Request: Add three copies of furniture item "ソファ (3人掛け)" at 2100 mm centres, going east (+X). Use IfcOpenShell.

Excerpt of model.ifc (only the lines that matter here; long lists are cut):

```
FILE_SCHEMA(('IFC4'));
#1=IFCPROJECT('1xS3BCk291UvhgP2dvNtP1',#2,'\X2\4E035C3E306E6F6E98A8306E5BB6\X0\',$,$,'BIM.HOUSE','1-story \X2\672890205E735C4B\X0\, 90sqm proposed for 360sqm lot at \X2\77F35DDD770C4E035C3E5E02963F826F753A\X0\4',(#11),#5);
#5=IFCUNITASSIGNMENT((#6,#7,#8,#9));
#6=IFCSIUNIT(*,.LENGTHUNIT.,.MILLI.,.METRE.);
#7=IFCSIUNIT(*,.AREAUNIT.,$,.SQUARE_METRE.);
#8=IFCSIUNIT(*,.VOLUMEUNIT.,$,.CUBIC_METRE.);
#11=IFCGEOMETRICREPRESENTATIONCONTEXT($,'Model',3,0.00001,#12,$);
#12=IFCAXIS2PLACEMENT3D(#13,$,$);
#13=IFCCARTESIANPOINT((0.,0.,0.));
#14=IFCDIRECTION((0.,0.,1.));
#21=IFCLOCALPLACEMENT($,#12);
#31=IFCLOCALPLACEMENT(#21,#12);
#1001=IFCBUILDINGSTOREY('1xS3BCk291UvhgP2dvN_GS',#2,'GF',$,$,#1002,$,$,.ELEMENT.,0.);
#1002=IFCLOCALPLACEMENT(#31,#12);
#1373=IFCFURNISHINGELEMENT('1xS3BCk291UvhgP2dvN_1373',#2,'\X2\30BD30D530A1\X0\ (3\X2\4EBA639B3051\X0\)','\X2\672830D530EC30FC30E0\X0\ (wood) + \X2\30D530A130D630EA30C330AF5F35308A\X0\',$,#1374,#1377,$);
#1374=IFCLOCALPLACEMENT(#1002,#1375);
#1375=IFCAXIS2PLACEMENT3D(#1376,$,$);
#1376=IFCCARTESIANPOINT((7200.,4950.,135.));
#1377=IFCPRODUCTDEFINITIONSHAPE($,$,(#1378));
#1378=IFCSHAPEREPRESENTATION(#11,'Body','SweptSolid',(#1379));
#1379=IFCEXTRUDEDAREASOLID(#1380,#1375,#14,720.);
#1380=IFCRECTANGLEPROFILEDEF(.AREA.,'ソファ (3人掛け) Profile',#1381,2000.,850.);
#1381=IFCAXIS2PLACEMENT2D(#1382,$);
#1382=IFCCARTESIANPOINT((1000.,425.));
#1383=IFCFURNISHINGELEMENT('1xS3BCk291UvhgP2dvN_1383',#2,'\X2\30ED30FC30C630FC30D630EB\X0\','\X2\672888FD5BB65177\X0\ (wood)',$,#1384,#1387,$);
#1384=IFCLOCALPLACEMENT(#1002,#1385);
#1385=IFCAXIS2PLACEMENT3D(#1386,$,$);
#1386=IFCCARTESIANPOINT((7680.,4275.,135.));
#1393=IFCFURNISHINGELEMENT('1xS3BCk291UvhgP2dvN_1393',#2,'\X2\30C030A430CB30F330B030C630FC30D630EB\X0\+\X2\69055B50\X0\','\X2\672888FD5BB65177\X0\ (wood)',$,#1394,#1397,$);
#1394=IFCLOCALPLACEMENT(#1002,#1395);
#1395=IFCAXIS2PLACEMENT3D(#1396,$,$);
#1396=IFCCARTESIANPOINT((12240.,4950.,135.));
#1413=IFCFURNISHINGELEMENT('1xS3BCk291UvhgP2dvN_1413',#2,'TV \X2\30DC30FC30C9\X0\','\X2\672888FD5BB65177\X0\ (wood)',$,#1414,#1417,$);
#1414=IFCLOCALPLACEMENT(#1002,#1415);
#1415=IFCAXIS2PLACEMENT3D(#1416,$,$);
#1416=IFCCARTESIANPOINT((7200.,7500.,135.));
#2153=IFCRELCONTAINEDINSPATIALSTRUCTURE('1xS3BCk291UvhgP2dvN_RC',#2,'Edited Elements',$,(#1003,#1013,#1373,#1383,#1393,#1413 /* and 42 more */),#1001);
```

```python
import numpy as np
import ifcopenshell
import ifcopenshell.api.geometry
import ifcopenshell.api.root
import ifcopenshell.util.element
import ifcopenshell.util.placement
import ifcopenshell.util.unit

model = ifcopenshell.open("model.ifc")
unit_scale = ifcopenshell.util.unit.calculate_unit_scale(model)


def reuse_history(source, copy):
    """copy_class also copies each property set's owner history, people and application; keep the originals."""
    for rel in copy.IsDefinedBy:
        if rel.is_a("IfcRelDefinesByProperties") and (history := rel.RelatingPropertyDefinition.OwnerHistory):
            rel.RelatingPropertyDefinition.OwnerHistory = source.OwnerHistory
            ifcopenshell.util.element.remove_deep2(model, history)


source = model.by_guid("1xS3BCk291UvhgP2dvN_1373")
base = ifcopenshell.util.placement.get_local_placement(source.ObjectPlacement)
step = np.array([1.0, 0.0, 0.0]) * 2.1 / unit_scale

for i in range(1, 4):
    copy = ifcopenshell.api.root.copy_class(model, product=source)
    copy.Representation = ifcopenshell.util.element.copy_deep(
        model, source.Representation, exclude=["IfcGeometricRepresentationContext", "IfcRepresentationMap"]
    )
    reuse_history(source, copy)
    matrix = base.copy()
    matrix[:3, 3] += i * step
    print("added at", matrix[:3, 3].round(3) + 0.0)
    ifcopenshell.api.geometry.edit_object_placement(model, product=copy, matrix=matrix, is_si=False)

model.write("model_updated.ifc")
```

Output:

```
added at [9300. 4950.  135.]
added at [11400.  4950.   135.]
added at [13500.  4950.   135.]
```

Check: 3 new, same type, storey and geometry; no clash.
